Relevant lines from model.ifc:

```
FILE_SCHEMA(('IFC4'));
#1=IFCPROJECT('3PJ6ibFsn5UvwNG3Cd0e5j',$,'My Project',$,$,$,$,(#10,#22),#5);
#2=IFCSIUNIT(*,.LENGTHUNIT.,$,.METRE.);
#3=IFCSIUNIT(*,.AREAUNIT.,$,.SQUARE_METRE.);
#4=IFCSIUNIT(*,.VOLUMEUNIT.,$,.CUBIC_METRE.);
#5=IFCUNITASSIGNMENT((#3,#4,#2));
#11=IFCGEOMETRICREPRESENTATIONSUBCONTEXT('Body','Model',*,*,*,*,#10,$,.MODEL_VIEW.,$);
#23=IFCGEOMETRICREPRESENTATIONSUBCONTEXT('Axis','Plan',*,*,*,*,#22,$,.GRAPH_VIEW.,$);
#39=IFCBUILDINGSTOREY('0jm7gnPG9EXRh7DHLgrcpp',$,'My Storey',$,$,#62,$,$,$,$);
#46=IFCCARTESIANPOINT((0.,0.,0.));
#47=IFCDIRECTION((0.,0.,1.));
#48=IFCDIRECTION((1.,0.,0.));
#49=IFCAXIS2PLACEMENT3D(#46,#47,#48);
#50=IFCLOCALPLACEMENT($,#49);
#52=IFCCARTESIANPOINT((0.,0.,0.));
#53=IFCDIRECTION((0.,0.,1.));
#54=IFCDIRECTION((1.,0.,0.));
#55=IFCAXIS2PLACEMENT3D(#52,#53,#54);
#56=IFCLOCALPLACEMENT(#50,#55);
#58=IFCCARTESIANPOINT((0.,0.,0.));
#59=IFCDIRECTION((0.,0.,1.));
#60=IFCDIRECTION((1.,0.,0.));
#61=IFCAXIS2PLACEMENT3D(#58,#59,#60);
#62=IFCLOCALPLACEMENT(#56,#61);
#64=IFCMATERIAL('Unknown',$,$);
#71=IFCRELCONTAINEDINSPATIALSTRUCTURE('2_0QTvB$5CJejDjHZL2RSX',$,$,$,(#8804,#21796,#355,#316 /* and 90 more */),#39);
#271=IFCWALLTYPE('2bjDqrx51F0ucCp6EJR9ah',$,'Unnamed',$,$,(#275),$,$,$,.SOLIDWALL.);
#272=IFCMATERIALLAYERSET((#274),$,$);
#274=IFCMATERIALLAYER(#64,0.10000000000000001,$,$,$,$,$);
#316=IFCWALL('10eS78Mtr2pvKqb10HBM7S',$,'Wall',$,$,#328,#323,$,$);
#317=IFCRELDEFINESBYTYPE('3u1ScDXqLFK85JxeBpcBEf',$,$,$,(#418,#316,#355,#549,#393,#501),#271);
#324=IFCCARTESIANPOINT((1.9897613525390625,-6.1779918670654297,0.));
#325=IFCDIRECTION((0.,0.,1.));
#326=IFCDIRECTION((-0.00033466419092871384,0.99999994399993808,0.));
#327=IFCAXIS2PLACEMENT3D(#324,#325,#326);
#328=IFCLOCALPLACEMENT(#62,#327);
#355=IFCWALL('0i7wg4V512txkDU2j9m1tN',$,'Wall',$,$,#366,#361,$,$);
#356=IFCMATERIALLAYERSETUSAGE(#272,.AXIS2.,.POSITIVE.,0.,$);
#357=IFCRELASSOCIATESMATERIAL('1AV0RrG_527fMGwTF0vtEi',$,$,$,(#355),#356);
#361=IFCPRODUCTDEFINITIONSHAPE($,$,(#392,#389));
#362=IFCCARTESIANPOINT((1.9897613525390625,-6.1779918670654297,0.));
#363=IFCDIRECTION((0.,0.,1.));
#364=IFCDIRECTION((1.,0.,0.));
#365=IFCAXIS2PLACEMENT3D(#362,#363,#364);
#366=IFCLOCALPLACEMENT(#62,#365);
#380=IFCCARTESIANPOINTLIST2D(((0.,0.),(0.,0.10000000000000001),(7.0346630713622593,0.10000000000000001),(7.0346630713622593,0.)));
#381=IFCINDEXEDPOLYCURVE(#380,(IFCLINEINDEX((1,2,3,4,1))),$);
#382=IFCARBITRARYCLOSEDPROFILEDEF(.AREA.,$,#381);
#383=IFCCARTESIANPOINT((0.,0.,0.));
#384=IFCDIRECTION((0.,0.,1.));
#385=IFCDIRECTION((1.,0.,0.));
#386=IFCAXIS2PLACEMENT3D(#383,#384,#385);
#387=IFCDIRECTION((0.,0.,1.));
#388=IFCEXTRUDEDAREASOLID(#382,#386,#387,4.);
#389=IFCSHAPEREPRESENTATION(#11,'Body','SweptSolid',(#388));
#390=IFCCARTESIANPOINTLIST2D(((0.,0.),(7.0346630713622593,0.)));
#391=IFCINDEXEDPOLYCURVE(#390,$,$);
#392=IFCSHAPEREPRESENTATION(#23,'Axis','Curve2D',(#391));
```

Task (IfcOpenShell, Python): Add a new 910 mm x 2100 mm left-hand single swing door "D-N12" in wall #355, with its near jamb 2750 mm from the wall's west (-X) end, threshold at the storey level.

```python
import numpy as np
import ifcopenshell
import ifcopenshell.api.feature
import ifcopenshell.api.geometry
import ifcopenshell.api.root
import ifcopenshell.api.spatial
import ifcopenshell.geom
import ifcopenshell.util.element
import ifcopenshell.util.placement
import ifcopenshell.util.representation
import ifcopenshell.util.shape
import ifcopenshell.util.unit

model = ifcopenshell.open("model.ifc")
unit_scale = ifcopenshell.util.unit.calculate_unit_scale(model)
settings = ifcopenshell.geom.settings()


def volume(element):
    """Net volume in cubic metres, openings subtracted."""
    shape = ifcopenshell.geom.create_shape(settings, element)
    return ifcopenshell.util.shape.get_volume(shape.geometry)


wall = model.by_guid("0i7wg4V512txkDU2j9m1tN")
storey = ifcopenshell.util.element.get_container(wall, ifc_class="IfcBuildingStorey")
context = ifcopenshell.util.representation.get_context(model, "Model", "Body", "MODEL_VIEW")
before = volume(wall)

width, height, from_end, sill = 0.91, 2.1, 2.75, 0.0  # metres

# The wall runs along its own X axis, and the end named is its -X end.
wall_shape = ifcopenshell.geom.create_shape(settings, wall)
x, y, z = ifcopenshell.util.shape.get_vertices(wall_shape.geometry).T
start = x.min() + from_end
face, thickness = float(y.min()), float(y.max() - y.min())
wall_matrix = ifcopenshell.util.placement.get_local_placement(wall.ObjectPlacement)
level = ifcopenshell.util.placement.get_local_placement(storey.ObjectPlacement)[2, 3]


def in_wall(x, y):
    """Placement at x, y metres in the wall's axes, at sill height."""
    matrix = wall_matrix.copy()
    matrix[:, 3] = wall_matrix @ np.array([x / unit_scale, y / unit_scale, 0.0, 1.0])
    matrix[2, 3] = level + sill / unit_scale
    return matrix


# Opening: a box that overshoots both wall faces by 50 mm.
opening = ifcopenshell.api.root.create_entity(model, ifc_class="IfcOpeningElement", predefined_type="OPENING")
box = ifcopenshell.api.geometry.add_wall_representation(
    model, context=context, length=width, height=height, thickness=thickness + 0.1
)
ifcopenshell.api.geometry.assign_representation(model, product=opening, representation=box)
ifcopenshell.api.geometry.edit_object_placement(model, product=opening, matrix=in_wall(start, face - 0.05), is_si=False)
ifcopenshell.api.feature.add_feature(model, feature=opening, element=wall)

door = ifcopenshell.api.root.create_entity(model, ifc_class="IfcDoor", name="D-N12", predefined_type="DOOR")
door.OverallWidth, door.OverallHeight = width / unit_scale, height / unit_scale
door.OperationType = "SINGLE_SWING_LEFT"
body = ifcopenshell.api.geometry.add_door_representation(
    model,
    context=context,
    overall_width=door.OverallWidth,
    overall_height=door.OverallHeight,
    operation_type="SINGLE_SWING_LEFT",
    lining_properties={"LiningDepth": thickness / unit_scale, "ThresholdDepth": thickness / unit_scale},
)
ifcopenshell.api.geometry.assign_representation(model, product=door, representation=body)
ifcopenshell.api.spatial.assign_container(model, products=[door], relating_structure=storey)
ifcopenshell.api.feature.add_filling(model, opening=opening, element=door)

# The lining spans the wall, so the door starts at the wall face.
ifcopenshell.api.geometry.edit_object_placement(model, product=door, matrix=in_wall(start, face), is_si=False)

after = volume(wall)

print(f"wall volume {before:.3f} -> {after:.3f} m3")

model.write("model_rev.ifc")
```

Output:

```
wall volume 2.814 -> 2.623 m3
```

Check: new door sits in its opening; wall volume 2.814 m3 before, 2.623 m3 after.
